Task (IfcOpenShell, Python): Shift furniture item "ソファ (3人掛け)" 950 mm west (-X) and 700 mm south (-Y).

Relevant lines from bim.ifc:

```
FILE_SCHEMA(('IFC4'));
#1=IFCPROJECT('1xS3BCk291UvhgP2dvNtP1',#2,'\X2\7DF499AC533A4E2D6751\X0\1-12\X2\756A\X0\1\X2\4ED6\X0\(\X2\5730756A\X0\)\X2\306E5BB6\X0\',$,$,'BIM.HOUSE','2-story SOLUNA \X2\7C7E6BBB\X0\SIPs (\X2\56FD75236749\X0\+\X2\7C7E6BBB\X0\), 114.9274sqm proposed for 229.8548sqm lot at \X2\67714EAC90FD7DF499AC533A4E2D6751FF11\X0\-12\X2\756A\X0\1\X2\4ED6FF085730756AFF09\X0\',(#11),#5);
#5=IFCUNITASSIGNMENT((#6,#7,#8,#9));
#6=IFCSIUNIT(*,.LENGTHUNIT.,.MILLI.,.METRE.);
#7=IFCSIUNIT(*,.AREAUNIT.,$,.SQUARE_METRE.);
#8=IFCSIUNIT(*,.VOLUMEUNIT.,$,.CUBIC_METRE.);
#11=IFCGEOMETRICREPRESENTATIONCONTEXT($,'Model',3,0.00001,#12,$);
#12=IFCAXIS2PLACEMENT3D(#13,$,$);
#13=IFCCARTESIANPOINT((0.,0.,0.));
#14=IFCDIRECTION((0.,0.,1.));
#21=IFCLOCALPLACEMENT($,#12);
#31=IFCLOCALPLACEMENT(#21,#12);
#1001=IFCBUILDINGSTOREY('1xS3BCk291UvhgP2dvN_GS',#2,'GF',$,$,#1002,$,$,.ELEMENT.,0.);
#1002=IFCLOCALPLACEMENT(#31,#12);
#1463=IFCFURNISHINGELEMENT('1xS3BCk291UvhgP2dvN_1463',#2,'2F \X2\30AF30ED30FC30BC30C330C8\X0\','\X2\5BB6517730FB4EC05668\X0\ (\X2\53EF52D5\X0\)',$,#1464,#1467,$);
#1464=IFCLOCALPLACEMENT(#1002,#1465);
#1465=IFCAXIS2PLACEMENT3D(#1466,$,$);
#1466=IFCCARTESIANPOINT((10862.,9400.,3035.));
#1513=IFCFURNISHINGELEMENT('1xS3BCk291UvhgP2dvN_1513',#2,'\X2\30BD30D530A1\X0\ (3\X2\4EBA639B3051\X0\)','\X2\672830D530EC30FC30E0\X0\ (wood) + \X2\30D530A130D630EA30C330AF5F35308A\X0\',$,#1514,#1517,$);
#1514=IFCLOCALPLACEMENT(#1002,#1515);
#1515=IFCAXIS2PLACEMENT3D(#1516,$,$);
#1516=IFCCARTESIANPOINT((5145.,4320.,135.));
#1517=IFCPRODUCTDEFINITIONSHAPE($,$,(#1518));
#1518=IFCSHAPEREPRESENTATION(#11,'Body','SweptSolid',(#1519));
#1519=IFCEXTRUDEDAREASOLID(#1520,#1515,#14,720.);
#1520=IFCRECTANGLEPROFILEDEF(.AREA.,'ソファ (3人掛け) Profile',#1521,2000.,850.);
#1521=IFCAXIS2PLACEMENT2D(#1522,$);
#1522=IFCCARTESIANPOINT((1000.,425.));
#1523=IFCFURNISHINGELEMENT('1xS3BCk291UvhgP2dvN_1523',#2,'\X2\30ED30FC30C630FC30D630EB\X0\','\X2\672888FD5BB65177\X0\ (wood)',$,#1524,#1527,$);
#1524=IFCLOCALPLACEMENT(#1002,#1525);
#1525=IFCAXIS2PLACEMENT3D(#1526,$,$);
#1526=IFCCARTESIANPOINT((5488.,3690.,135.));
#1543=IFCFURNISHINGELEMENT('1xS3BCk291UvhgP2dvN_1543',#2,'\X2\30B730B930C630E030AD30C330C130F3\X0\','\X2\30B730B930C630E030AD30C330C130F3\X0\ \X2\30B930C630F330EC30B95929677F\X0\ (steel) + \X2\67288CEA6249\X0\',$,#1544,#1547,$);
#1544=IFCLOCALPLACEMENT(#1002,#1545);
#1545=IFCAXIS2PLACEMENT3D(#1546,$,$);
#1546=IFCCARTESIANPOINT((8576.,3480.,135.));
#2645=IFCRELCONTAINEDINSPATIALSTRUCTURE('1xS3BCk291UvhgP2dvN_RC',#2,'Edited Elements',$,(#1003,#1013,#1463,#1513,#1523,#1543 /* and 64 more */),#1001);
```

```python
import ifcopenshell
import ifcopenshell.api.geometry
import ifcopenshell.util.placement
import ifcopenshell.util.unit

model = ifcopenshell.open("bim.ifc")
unit_scale = ifcopenshell.util.unit.calculate_unit_scale(model)

item = model.by_guid("1xS3BCk291UvhgP2dvN_1513")
matrix = ifcopenshell.util.placement.get_local_placement(item.ObjectPlacement)
matrix[0, 3] -= 0.95 / unit_scale
matrix[1, 3] -= 0.7 / unit_scale
ifcopenshell.api.geometry.edit_object_placement(model, product=item, matrix=matrix, is_si=False)

print(ifcopenshell.util.placement.get_local_placement(item.ObjectPlacement).round(3) + 0.0)

model.write("bim-out.ifc")
```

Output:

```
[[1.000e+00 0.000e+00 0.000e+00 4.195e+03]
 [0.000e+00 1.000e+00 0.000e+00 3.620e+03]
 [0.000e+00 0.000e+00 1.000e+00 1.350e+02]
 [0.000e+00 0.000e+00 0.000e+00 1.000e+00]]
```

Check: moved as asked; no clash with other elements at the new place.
